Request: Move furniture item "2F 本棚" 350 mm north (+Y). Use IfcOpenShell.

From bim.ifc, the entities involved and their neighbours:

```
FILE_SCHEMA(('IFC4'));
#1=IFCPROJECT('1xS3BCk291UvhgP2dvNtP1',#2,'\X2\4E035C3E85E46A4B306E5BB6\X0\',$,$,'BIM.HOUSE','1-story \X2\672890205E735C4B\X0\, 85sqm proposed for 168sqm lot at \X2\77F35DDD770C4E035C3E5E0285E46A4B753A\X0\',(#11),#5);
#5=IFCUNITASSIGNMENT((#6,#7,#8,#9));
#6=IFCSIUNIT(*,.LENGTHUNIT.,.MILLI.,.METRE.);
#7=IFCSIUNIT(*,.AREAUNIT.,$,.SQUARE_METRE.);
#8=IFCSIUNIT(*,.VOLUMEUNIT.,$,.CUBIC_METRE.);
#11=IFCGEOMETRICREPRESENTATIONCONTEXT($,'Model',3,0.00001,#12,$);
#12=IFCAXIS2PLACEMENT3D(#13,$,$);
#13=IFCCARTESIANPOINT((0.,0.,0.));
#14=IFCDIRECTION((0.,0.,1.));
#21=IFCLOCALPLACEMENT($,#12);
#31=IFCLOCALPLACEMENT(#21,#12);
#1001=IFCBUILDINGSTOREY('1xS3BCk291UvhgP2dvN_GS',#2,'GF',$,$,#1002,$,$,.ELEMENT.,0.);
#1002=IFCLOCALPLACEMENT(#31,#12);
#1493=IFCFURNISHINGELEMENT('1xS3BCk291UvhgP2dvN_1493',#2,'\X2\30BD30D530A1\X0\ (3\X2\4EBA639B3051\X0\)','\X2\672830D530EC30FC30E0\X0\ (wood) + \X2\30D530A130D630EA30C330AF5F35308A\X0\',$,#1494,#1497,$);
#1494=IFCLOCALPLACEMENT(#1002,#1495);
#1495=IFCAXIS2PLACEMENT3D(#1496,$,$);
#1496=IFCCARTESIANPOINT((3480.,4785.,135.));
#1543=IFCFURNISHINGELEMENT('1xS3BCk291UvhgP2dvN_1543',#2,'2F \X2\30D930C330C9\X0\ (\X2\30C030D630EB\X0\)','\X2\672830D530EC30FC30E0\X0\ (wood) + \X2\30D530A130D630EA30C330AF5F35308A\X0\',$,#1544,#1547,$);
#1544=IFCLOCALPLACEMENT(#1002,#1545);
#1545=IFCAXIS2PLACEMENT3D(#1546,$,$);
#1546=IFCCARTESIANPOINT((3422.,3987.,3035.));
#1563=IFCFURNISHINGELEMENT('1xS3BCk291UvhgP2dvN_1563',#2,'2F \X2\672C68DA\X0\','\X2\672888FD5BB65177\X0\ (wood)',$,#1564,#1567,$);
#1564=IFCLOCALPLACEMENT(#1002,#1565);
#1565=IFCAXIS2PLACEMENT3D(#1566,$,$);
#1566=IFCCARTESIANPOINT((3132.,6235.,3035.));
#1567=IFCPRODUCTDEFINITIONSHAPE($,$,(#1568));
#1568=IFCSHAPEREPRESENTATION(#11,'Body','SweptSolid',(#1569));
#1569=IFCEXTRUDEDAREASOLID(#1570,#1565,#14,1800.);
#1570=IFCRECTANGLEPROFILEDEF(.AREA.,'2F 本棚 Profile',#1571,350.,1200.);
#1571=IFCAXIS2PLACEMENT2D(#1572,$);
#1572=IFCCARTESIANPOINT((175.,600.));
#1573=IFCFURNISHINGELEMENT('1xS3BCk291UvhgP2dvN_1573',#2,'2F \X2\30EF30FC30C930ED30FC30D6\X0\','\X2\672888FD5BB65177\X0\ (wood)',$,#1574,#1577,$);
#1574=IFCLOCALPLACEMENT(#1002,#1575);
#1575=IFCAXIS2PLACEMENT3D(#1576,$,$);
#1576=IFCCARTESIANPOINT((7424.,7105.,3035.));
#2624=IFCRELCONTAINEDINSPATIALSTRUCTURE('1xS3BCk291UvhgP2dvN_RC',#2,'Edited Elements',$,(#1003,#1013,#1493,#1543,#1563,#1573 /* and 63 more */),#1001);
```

```python
import ifcopenshell
import ifcopenshell.api.geometry
import ifcopenshell.util.placement

model = ifcopenshell.open("bim.ifc")

item = model.by_guid("1xS3BCk291UvhgP2dvN_1563")
matrix = ifcopenshell.util.placement.get_local_placement(item.ObjectPlacement)
matrix[1, 3] += 350.0
ifcopenshell.api.geometry.edit_object_placement(model, product=item, matrix=matrix, is_si=False)

print(ifcopenshell.util.placement.get_local_placement(item.ObjectPlacement).round(3) + 0.0)

model.write("bim-out.ifc")
```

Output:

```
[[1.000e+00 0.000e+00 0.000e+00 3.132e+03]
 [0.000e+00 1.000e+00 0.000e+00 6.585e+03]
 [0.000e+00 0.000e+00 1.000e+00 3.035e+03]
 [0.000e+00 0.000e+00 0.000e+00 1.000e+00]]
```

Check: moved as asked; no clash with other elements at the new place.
